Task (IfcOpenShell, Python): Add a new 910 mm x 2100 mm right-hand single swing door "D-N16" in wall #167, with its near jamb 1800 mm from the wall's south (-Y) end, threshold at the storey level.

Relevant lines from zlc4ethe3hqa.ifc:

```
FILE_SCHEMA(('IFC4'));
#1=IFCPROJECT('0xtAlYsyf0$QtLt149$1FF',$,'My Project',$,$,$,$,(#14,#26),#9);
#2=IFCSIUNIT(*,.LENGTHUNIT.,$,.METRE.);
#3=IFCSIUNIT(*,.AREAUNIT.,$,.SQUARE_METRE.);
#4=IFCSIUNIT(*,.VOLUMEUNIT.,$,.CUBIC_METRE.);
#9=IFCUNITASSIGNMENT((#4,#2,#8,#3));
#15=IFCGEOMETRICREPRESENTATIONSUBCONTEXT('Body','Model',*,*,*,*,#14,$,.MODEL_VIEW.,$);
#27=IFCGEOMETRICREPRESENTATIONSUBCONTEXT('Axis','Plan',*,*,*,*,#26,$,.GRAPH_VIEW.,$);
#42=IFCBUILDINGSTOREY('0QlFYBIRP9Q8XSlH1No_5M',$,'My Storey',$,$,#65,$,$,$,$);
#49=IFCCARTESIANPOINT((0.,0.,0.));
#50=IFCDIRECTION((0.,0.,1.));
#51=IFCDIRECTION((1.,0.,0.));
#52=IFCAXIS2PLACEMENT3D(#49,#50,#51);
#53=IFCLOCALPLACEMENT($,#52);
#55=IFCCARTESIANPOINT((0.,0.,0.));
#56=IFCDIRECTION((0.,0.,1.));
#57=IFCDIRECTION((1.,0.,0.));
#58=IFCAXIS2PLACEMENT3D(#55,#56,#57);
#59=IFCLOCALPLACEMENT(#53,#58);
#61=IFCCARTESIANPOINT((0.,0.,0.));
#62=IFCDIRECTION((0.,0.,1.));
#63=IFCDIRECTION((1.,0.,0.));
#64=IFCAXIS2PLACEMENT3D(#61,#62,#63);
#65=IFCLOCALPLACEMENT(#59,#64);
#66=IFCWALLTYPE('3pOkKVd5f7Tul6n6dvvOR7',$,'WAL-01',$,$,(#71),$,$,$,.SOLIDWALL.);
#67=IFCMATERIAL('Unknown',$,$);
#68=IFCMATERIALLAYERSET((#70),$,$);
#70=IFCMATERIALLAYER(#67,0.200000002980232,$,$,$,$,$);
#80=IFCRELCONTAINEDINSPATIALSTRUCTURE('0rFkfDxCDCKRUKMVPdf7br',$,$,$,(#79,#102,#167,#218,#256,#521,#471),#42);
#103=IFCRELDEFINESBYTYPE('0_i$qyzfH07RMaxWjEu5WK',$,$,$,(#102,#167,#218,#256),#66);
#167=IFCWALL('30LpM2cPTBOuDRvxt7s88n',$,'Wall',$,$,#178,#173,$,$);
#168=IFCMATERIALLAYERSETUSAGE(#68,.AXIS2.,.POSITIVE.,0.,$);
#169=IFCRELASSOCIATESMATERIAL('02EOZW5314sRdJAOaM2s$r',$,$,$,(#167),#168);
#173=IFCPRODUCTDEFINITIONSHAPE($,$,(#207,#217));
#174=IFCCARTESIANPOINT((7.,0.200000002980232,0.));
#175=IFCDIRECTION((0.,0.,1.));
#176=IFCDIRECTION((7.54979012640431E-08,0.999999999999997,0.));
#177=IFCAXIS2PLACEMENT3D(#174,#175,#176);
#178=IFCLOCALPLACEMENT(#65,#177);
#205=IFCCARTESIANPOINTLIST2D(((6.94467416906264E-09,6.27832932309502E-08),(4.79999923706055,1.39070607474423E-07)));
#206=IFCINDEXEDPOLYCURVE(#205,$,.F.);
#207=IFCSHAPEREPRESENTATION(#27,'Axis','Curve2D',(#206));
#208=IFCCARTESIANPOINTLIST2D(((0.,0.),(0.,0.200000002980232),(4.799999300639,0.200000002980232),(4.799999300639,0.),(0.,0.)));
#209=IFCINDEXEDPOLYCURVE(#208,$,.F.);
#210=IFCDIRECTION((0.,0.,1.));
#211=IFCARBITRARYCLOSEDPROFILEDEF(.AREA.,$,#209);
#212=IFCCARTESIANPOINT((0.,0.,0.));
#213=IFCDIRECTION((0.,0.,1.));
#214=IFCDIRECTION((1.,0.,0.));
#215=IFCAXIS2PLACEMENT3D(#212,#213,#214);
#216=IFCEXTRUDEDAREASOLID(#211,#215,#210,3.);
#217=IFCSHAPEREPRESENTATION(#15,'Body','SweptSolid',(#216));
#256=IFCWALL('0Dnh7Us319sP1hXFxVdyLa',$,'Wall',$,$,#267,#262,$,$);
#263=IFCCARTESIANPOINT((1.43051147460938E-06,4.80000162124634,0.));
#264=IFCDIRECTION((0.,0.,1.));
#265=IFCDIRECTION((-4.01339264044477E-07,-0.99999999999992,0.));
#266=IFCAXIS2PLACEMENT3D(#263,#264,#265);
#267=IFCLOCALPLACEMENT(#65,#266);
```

```python
import numpy as np
import ifcopenshell
import ifcopenshell.api.feature
import ifcopenshell.api.geometry
import ifcopenshell.api.root
import ifcopenshell.api.spatial
import ifcopenshell.geom
import ifcopenshell.util.element
import ifcopenshell.util.placement
import ifcopenshell.util.representation
import ifcopenshell.util.shape
import ifcopenshell.util.unit

model = ifcopenshell.open("zlc4ethe3hqa.ifc")
unit_scale = ifcopenshell.util.unit.calculate_unit_scale(model)
settings = ifcopenshell.geom.settings()


def volume(element):
    """Net volume in cubic metres, openings subtracted."""
    shape = ifcopenshell.geom.create_shape(settings, element)
    return ifcopenshell.util.shape.get_volume(shape.geometry)


wall = model.by_id(167)
storey = ifcopenshell.util.element.get_container(wall, ifc_class="IfcBuildingStorey")
context = ifcopenshell.util.representation.get_context(model, "Model", "Body", "MODEL_VIEW")
before = volume(wall)

width, height, from_end, sill = 0.91, 2.1, 1.8, 0.0  # metres

# The wall runs along its own X axis, and the end named is its -X end.
wall_shape = ifcopenshell.geom.create_shape(settings, wall)
x, y, z = ifcopenshell.util.shape.get_vertices(wall_shape.geometry).T
start = x.min() + from_end
face, thickness = float(y.min()), float(y.max() - y.min())
wall_matrix = ifcopenshell.util.placement.get_local_placement(wall.ObjectPlacement)
level = ifcopenshell.util.placement.get_local_placement(storey.ObjectPlacement)[2, 3]


def in_wall(x, y):
    """Placement at x, y metres in the wall's axes, at sill height."""
    matrix = wall_matrix.copy()
    matrix[:, 3] = wall_matrix @ np.array([x / unit_scale, y / unit_scale, 0.0, 1.0])
    matrix[2, 3] = level + sill / unit_scale
    return matrix


# Opening: a box that overshoots both wall faces by 50 mm.
opening = ifcopenshell.api.root.create_entity(model, ifc_class="IfcOpeningElement", predefined_type="OPENING")
box = ifcopenshell.api.geometry.add_wall_representation(
    model, context=context, length=width, height=height, thickness=thickness + 0.1
)
ifcopenshell.api.geometry.assign_representation(model, product=opening, representation=box)
ifcopenshell.api.geometry.edit_object_placement(model, product=opening, matrix=in_wall(start, face - 0.05), is_si=False)
ifcopenshell.api.feature.add_feature(model, feature=opening, element=wall)

door = ifcopenshell.api.root.create_entity(model, ifc_class="IfcDoor", name="D-N16", predefined_type="DOOR")
door.OverallWidth, door.OverallHeight = width / unit_scale, height / unit_scale
door.OperationType = "SINGLE_SWING_RIGHT"
body = ifcopenshell.api.geometry.add_door_representation(
    model,
    context=context,
    overall_width=door.OverallWidth,
    overall_height=door.OverallHeight,
    operation_type="SINGLE_SWING_RIGHT",
    lining_properties={"LiningDepth": thickness / unit_scale, "ThresholdDepth": thickness / unit_scale},
)
ifcopenshell.api.geometry.assign_representation(model, product=door, representation=body)
ifcopenshell.api.spatial.assign_container(model, products=[door], relating_structure=storey)
ifcopenshell.api.feature.add_filling(model, opening=opening, element=door)

# The lining spans the wall, so the door starts at the wall face.
ifcopenshell.api.geometry.edit_object_placement(model, product=door, matrix=in_wall(start, face), is_si=False)

after = volume(wall)

print(f"wall volume {before:.3f} -> {after:.3f} m3")

model.write("zlc4ethe3hqa_edited.ifc")
```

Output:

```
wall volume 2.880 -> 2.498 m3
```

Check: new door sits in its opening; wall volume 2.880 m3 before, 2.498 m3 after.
